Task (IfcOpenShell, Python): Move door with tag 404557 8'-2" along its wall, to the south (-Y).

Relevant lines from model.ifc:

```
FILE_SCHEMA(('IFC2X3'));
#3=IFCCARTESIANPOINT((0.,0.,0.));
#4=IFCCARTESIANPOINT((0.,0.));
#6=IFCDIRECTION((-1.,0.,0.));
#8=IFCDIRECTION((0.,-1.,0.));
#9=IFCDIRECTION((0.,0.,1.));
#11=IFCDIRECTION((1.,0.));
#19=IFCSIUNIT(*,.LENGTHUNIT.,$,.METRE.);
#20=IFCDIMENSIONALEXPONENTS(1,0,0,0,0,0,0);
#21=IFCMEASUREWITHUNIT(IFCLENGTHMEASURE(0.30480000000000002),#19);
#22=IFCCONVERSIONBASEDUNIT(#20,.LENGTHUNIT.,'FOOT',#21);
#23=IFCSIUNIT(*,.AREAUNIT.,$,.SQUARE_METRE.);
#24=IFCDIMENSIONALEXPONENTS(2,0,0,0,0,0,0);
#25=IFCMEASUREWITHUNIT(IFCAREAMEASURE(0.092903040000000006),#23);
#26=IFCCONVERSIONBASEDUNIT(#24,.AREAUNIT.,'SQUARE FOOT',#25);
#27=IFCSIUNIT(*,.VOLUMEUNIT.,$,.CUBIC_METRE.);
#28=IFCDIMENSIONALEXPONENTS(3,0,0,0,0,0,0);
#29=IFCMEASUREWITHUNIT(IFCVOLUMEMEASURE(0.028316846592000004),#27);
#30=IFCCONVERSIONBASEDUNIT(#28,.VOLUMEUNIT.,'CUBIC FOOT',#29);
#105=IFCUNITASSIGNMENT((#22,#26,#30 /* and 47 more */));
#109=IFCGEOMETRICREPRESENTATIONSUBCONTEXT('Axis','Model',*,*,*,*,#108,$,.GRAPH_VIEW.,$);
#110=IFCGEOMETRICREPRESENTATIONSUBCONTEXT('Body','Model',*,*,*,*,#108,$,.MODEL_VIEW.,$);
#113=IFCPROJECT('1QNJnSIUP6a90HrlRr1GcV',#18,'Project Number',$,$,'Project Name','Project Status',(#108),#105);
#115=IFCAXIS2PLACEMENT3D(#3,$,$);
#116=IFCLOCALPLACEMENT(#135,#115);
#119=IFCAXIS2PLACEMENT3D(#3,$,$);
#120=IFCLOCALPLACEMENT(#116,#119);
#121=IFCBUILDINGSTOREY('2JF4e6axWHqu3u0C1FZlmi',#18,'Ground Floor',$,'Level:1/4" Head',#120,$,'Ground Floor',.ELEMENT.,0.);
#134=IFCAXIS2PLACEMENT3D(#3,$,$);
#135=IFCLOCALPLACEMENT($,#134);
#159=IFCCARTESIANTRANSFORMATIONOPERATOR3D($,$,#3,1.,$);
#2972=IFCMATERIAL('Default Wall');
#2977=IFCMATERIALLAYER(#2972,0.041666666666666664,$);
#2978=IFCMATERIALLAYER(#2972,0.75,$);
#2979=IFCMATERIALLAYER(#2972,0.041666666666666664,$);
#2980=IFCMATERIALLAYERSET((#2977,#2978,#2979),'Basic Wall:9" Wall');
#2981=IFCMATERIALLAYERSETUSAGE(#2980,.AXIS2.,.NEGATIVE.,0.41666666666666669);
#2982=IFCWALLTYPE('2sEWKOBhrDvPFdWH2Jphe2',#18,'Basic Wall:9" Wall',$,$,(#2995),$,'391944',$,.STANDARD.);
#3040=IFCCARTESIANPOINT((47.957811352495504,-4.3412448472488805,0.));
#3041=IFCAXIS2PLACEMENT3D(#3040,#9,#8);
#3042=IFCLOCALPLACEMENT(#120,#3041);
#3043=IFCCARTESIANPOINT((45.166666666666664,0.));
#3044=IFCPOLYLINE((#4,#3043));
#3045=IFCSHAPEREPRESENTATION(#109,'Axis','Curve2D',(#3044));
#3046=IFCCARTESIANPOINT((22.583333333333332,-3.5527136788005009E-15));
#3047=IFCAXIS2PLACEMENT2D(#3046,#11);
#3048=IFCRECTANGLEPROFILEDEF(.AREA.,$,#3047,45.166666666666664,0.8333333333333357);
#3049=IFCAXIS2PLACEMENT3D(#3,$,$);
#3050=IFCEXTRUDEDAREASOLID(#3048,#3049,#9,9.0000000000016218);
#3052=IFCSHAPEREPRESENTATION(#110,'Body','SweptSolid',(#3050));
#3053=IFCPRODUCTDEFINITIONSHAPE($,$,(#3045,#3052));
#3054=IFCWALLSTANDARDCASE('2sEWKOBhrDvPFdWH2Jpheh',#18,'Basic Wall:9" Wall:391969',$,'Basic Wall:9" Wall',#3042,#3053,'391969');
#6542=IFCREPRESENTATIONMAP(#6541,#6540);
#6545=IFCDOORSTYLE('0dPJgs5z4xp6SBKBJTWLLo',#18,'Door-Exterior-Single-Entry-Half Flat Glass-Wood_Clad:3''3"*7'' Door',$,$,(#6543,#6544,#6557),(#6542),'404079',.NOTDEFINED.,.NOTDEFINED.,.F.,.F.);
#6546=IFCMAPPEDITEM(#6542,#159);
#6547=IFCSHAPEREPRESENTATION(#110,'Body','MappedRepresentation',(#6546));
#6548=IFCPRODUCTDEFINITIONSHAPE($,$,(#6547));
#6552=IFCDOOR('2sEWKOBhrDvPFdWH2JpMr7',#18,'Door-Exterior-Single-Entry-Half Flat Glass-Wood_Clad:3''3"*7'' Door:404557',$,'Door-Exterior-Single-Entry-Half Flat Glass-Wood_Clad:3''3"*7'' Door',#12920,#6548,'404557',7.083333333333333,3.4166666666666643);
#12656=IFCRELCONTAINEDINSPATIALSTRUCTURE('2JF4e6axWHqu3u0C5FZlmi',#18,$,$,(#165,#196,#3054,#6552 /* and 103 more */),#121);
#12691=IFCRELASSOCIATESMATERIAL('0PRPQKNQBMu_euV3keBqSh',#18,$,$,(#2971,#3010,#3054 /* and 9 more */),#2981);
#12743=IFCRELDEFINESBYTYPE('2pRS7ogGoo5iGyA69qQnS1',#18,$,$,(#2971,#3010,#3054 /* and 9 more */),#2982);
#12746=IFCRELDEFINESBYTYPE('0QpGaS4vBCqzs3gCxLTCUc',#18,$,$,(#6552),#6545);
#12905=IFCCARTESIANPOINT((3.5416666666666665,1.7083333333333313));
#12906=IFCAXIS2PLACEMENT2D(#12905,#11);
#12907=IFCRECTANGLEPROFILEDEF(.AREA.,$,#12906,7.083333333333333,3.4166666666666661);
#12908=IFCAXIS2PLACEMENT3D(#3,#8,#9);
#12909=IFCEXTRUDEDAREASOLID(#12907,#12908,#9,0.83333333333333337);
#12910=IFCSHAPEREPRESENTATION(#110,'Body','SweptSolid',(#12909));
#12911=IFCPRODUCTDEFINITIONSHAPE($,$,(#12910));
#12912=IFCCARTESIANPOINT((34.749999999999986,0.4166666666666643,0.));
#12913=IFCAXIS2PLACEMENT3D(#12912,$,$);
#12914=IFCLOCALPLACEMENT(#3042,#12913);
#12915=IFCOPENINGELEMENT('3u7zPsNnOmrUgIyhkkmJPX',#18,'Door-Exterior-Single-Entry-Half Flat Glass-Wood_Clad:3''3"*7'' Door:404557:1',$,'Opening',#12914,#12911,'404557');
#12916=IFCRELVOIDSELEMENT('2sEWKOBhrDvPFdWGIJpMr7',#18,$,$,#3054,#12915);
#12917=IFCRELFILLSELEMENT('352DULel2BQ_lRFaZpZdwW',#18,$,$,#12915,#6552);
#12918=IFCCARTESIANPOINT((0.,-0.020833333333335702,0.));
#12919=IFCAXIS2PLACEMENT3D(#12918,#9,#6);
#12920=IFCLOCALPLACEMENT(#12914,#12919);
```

```python
import ifcopenshell
import ifcopenshell.api.geometry
import ifcopenshell.util.placement
import ifcopenshell.util.unit

model = ifcopenshell.open("model.ifc")
unit_scale = ifcopenshell.util.unit.calculate_unit_scale(model)

door = model.by_guid("2sEWKOBhrDvPFdWH2JpMr7")
opening = door.FillsVoids[0].RelatingOpeningElement
wall = opening.VoidsElements[0].RelatingBuildingElement

wall_matrix = ifcopenshell.util.placement.get_local_placement(wall.ObjectPlacement)
shift = wall_matrix[:3, 0] * 98 * 0.0254 / unit_scale
before = ifcopenshell.util.placement.get_local_placement(door.ObjectPlacement)[:3, 3].copy()

# The door is placed relative to its opening, so it follows when the opening moves.
matrix = ifcopenshell.util.placement.get_local_placement(opening.ObjectPlacement)
matrix[:3, 3] += shift
ifcopenshell.api.geometry.edit_object_placement(
    model, product=opening, matrix=matrix, is_si=False, should_transform_children=True
)

after = ifcopenshell.util.placement.get_local_placement(door.ObjectPlacement)[:3, 3]
print("door moved by", (after - before).round(3) + 0.0)

model.write("model_v2.ifc")
```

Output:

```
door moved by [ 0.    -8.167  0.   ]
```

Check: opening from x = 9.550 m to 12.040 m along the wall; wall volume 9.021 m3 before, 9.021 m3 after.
